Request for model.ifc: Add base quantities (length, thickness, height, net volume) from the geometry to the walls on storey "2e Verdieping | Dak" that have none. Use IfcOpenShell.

First a look at what the model holds.

```python
import ifcopenshell
import ifcopenshell.util.element
import ifcopenshell.util.unit

model = ifcopenshell.open("model.ifc")
print(model.schema)
for unit_type in ("LENGTHUNIT", "AREAUNIT", "VOLUMEUNIT"):
    print(unit_type, ifcopenshell.util.unit.calculate_unit_scale(model, unit_type))
storey = next(s for s in model.by_type("IfcBuildingStorey") if s.Name == "2e Verdieping | Dak")
walls = [e for e in ifcopenshell.util.element.get_decomposition(storey) if e.is_a("IfcWall")]
for e in sorted(walls, key=lambda e: e.id()):
    print(e.id(), e.is_a(), e.Name, list(ifcopenshell.util.element.get_psets(e, qtos_only=True)), sep=" | ")
```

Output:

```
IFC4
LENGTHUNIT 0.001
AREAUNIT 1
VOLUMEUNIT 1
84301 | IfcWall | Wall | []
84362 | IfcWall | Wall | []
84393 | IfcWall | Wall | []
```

```python
import ifcopenshell
import ifcopenshell.api.pset
import ifcopenshell.geom
import ifcopenshell.util.element
import ifcopenshell.util.shape
import ifcopenshell.util.unit

model = ifcopenshell.open("model.ifc")
unit_scale = ifcopenshell.util.unit.calculate_unit_scale(model)
volume_scale = ifcopenshell.util.unit.calculate_unit_scale(model, "VOLUMEUNIT")
settings = ifcopenshell.geom.settings()

storey = next(s for s in model.by_type("IfcBuildingStorey") if s.Name == "2e Verdieping | Dak")
walls = [e for e in ifcopenshell.util.element.get_decomposition(storey) if e.is_a("IfcWall")]

for e in sorted(walls, key=lambda e: e.id()):
    if ifcopenshell.util.element.get_psets(e, qtos_only=True, should_inherit=False):
        continue
    # Geometry comes back in metres, in the element's own axes.
    shape = ifcopenshell.geom.create_shape(settings, e)
    values = {
        "Length": ifcopenshell.util.shape.get_x(shape.geometry) / unit_scale,
        "Width": ifcopenshell.util.shape.get_y(shape.geometry) / unit_scale,
        "Height": ifcopenshell.util.shape.get_z(shape.geometry) / unit_scale,
        "NetVolume": ifcopenshell.util.shape.get_volume(shape.geometry) / volume_scale,
    }
    qto = ifcopenshell.api.pset.add_qto(model, product=e, name="Qto_WallBaseQuantities")
    ifcopenshell.api.pset.edit_qto(model, qto=qto, properties=values)
    print(e.id(), {k: round(v, 3) for k, v in values.items()})

model.write("model_edited.ifc")
```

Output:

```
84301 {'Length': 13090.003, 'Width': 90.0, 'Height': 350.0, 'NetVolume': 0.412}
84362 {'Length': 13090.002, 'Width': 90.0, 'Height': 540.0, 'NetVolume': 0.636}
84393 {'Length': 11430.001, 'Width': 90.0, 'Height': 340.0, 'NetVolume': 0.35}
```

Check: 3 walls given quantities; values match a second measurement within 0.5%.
